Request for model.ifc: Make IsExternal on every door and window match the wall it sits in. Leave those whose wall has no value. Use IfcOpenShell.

First a look at what the model holds.

```python
import ifcopenshell
import ifcopenshell.util.element

model = ifcopenshell.open("model.ifc")
print(model.schema)
seen = {}
for e in model.by_type("IfcDoor") + model.by_type("IfcWindow"):
    if not e.FillsVoids:
        continue
    host = e.FillsVoids[0].RelatingOpeningElement.VoidsElements[0].RelatingBuildingElement
    own = ifcopenshell.util.element.get_pset(e, f"Pset_{e.is_a()[3:].removesuffix('StandardCase')}Common", "IsExternal")
    wall = ifcopenshell.util.element.get_pset(host, "Pset_WallCommon", "IsExternal")
    seen[e.is_a(), own, wall] = seen.get((e.is_a(), own, wall), 0) + 1
for (cls, own, wall), count in sorted(seen.items(), key=str):
    print(count, cls, "IsExternal:", own, "| host wall:", wall)
```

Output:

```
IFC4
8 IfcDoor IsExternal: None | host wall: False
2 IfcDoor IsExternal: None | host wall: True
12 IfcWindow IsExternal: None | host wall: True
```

```python
import ifcopenshell
import ifcopenshell.api.pset
import ifcopenshell.util.element

model = ifcopenshell.open("model.ifc")

count = 0
for ifc_class, pset_name in (("IfcDoor", "Pset_DoorCommon"), ("IfcWindow", "Pset_WindowCommon")):
    for e in model.by_type(ifc_class):
        if not e.FillsVoids:
            continue
        host = e.FillsVoids[0].RelatingOpeningElement.VoidsElements[0].RelatingBuildingElement
        external = ifcopenshell.util.element.get_pset(host, "Pset_WallCommon", "IsExternal")
        if external is None or ifcopenshell.util.element.get_pset(e, pset_name, "IsExternal") == external:
            continue
        pset = ifcopenshell.api.pset.add_pset(model, product=e, name=pset_name)
        ifcopenshell.api.pset.edit_pset(model, pset=pset, properties={"IsExternal": external})
        count += 1

print(count, "updated")

model.write("model_rev.ifc")
```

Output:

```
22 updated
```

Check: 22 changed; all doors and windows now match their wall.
